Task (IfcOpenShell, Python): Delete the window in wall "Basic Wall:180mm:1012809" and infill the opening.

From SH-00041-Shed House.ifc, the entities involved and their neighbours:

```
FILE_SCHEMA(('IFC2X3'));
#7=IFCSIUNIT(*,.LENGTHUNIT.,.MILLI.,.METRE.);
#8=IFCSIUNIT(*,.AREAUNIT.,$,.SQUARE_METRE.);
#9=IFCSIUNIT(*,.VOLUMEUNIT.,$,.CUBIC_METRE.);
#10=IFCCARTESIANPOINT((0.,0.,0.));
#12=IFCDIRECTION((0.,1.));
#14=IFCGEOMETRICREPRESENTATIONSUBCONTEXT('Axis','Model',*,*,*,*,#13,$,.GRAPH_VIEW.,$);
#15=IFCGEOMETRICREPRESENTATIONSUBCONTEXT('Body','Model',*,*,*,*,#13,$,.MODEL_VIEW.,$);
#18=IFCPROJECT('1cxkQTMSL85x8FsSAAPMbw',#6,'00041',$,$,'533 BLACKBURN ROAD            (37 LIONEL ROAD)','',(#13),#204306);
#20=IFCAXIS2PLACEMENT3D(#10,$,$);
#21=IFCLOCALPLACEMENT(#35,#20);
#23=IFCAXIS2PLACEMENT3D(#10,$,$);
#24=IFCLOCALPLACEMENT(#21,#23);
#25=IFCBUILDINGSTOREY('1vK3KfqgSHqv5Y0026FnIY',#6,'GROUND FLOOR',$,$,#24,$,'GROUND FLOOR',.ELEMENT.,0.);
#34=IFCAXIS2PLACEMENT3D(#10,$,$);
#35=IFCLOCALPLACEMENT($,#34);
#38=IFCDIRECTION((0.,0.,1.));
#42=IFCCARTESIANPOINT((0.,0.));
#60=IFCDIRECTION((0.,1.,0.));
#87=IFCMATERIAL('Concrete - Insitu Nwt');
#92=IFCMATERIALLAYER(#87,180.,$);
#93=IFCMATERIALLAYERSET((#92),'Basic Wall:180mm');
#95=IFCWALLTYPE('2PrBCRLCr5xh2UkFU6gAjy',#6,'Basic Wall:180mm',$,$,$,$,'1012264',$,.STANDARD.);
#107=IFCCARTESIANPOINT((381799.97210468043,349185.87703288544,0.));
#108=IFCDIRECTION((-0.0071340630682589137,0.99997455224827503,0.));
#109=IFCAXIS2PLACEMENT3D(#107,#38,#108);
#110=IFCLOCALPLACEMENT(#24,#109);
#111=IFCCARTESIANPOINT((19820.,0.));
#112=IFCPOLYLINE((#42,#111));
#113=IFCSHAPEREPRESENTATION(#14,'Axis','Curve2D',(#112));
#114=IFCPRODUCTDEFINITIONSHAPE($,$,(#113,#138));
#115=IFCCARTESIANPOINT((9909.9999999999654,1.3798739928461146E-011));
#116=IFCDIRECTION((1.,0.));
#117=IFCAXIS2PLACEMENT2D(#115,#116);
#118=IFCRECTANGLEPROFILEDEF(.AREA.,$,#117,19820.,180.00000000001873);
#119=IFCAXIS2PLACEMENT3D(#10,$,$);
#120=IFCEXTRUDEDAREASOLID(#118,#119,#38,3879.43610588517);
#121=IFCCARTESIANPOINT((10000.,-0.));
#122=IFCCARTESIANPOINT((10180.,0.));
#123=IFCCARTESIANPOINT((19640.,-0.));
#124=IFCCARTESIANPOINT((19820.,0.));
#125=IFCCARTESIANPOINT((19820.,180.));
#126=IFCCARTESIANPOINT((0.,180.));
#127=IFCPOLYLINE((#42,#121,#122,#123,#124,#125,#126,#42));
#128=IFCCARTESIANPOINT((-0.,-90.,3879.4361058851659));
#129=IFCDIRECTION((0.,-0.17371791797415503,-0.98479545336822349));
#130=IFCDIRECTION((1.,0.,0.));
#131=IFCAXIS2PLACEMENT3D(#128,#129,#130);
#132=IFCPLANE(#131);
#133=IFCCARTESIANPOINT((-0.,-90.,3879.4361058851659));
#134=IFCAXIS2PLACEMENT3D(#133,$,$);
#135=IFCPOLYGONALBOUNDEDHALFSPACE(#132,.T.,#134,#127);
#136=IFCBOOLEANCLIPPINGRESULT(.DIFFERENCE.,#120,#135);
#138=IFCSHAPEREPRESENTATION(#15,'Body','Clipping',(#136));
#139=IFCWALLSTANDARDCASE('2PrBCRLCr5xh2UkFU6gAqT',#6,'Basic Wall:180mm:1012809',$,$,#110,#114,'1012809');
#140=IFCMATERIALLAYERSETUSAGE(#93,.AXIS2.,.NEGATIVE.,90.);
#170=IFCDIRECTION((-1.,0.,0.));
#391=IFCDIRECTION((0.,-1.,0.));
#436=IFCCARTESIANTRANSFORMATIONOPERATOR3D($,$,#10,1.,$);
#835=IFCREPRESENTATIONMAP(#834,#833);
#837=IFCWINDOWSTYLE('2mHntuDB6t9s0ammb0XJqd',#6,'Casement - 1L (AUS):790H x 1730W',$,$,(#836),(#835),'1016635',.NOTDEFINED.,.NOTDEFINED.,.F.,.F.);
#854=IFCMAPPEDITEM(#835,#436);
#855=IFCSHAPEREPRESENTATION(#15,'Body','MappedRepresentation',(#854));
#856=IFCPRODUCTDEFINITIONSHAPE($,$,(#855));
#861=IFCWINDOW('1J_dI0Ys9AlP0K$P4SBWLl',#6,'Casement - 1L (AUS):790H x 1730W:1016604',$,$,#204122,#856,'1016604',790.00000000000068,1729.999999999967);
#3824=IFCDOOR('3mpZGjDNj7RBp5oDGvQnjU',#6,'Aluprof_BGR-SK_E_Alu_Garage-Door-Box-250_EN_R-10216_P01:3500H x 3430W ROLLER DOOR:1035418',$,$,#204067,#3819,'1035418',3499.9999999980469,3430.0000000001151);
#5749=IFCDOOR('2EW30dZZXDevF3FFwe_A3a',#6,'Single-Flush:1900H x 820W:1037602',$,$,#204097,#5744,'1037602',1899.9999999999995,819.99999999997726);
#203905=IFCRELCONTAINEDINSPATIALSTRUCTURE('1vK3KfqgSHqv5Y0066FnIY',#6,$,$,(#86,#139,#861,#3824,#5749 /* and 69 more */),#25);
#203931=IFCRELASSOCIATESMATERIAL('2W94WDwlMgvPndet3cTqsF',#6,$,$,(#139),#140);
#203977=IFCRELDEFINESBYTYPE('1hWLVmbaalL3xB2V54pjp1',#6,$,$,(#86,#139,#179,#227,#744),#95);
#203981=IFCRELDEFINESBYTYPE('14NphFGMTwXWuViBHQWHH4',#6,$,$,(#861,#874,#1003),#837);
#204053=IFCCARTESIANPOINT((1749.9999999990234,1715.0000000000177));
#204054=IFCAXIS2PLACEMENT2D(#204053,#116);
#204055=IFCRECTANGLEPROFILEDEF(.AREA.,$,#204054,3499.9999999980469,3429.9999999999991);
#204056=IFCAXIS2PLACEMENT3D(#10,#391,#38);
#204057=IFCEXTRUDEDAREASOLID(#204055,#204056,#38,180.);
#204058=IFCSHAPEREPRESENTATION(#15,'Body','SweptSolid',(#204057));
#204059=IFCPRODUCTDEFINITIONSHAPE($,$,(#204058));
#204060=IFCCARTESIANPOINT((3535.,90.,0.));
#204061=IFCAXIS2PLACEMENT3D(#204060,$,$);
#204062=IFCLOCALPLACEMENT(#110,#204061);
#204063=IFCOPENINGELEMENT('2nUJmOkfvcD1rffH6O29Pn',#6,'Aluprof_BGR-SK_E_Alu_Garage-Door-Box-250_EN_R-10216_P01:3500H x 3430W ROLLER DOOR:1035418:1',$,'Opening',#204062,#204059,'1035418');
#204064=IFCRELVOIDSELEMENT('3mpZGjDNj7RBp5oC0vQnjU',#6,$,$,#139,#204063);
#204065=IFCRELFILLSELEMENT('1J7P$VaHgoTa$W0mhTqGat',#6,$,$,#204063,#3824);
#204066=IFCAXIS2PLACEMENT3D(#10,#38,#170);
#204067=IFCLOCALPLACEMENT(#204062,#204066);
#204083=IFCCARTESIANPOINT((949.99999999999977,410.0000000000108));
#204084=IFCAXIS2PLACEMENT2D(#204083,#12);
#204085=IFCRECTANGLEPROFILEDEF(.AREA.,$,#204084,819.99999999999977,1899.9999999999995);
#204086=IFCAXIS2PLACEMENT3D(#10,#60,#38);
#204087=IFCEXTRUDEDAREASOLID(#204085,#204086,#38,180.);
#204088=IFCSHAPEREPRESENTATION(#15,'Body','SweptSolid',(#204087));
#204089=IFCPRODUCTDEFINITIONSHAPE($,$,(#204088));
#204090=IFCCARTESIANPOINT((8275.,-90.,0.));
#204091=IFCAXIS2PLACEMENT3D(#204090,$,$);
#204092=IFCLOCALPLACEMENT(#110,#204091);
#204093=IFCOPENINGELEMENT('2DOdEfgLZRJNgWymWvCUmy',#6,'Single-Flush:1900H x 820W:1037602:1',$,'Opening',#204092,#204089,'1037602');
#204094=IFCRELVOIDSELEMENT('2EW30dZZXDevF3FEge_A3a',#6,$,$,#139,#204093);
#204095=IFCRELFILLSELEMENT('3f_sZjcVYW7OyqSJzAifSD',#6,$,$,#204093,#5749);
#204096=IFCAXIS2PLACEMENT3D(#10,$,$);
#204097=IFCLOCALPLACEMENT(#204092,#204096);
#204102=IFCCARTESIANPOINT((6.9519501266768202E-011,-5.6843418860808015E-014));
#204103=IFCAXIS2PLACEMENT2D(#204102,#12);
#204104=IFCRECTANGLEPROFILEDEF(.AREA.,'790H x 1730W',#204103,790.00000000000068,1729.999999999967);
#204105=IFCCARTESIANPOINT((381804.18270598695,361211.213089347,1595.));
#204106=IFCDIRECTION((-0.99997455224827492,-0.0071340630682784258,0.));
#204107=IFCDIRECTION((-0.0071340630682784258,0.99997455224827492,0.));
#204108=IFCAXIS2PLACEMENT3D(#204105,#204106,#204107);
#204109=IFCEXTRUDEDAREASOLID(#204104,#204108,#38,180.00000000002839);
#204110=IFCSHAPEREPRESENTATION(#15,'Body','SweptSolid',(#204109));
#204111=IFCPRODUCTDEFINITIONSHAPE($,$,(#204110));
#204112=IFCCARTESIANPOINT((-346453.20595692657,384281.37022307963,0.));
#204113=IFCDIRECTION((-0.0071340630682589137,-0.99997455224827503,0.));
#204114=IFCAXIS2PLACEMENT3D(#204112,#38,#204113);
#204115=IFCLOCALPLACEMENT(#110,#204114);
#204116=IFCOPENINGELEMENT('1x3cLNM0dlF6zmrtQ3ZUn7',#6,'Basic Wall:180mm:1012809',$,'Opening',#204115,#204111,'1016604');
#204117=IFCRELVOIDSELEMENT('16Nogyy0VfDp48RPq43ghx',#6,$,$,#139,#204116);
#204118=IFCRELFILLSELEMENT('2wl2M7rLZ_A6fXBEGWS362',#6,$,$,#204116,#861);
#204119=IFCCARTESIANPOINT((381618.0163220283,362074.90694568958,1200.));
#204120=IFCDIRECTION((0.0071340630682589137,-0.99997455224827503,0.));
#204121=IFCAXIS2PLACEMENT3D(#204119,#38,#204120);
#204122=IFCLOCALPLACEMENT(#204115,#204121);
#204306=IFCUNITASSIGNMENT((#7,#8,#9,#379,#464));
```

```python
import ifcopenshell
import ifcopenshell.api.feature
import ifcopenshell.api.root
import ifcopenshell.geom
import ifcopenshell.util.shape

model = ifcopenshell.open("SH-00041-Shed House.ifc")
settings = ifcopenshell.geom.settings()


def volume(element):
    """Net volume in cubic metres, openings subtracted."""
    shape = ifcopenshell.geom.create_shape(settings, element)
    return ifcopenshell.util.shape.get_volume(shape.geometry)


window = model.by_guid("1J_dI0Ys9AlP0K$P4SBWLl")
opening = window.FillsVoids[0].RelatingOpeningElement
wall = opening.VoidsElements[0].RelatingBuildingElement
before = volume(wall)

ifcopenshell.api.root.remove_product(model, product=window)
ifcopenshell.api.feature.remove_feature(model, feature=opening)

after = volume(wall)

print(f"wall volume {before:.3f} -> {after:.3f} m3")

model.write("SH-00041-Shed House_updated.ifc")
```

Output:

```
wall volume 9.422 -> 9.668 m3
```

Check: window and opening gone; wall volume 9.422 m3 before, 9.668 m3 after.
